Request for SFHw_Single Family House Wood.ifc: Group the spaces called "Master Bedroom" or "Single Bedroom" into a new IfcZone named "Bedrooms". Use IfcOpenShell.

First a look at what the model holds.

```python
import ifcopenshell

model = ifcopenshell.open("SFHw_Single Family House Wood.ifc")
print(model.schema)
seen = {}
for space in model.by_type("IfcSpace"):
    seen[space.LongName] = seen.get(space.LongName, 0) + 1
for name, count in sorted(seen.items(), key=str):
    print(count, "x", name)
print("zones:", [z.Name for z in model.by_type("IfcZone")][:20])
```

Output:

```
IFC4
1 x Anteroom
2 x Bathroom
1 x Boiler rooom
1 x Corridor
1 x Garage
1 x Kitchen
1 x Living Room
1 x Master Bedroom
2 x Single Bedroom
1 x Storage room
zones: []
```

```python
import ifcopenshell
import ifcopenshell.api.group
import ifcopenshell.api.root

model = ifcopenshell.open("SFHw_Single Family House Wood.ifc")

names = {"Master Bedroom", "Single Bedroom"}
spaces = [s for s in model.by_type("IfcSpace") if s.LongName in names]

zone = ifcopenshell.api.root.create_entity(model, ifc_class="IfcZone", name="Bedrooms")
ifcopenshell.api.group.assign_group(model, products=spaces, group=zone)
print(len(spaces), "spaces in", zone.Name)

model.write("SFHw_Single Family House Wood_rev.ifc")
```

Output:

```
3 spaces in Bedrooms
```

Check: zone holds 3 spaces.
